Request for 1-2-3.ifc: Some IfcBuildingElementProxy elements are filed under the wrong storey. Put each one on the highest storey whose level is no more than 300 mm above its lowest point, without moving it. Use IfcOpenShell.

First a look at what the model holds.

```python
import ifcopenshell
import ifcopenshell.util.element
import ifcopenshell.util.placement

model = ifcopenshell.open("1-2-3.ifc")
print(model.schema)
for storey in model.by_type("IfcBuildingStorey"):
    level = ifcopenshell.util.placement.get_storey_elevation(storey)
    count = sum(e.is_a("IfcBuildingElementProxy") for e in ifcopenshell.util.element.get_contained(storey))
    print(storey.id(), storey.Name, round(level, 3), count, sep=" | ")
```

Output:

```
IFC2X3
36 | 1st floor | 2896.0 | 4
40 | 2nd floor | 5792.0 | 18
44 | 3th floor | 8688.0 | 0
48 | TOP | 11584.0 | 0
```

```python
import ifcopenshell
import ifcopenshell.api.spatial
import ifcopenshell.geom
import ifcopenshell.util.element
import ifcopenshell.util.placement
import ifcopenshell.util.shape
import ifcopenshell.util.unit

model = ifcopenshell.open("1-2-3.ifc")
unit_scale = ifcopenshell.util.unit.calculate_unit_scale(model)
settings = ifcopenshell.geom.settings()

levels = sorted(
    ((ifcopenshell.util.placement.get_storey_elevation(s) * unit_scale, s) for s in model.by_type("IfcBuildingStorey")),
    key=lambda pair: pair[0],
)

for e in model.by_type("IfcBuildingElementProxy"):
    current = e.ContainedInStructure[0].RelatingStructure if e.ContainedInStructure else None
    if current is None or not current.is_a("IfcBuildingStorey"):
        continue
    shape = ifcopenshell.geom.create_shape(settings, e)
    bottom = ifcopenshell.util.shape.get_shape_bottom_elevation(shape, shape.geometry)
    below = [s for level, s in levels if level <= bottom + 0.3]
    storey = below[-1] if below else levels[0][1]
    if storey != current:
        # assign_container keeps the world position.
        ifcopenshell.api.spatial.assign_container(model, products=[e], relating_structure=storey)
        print(e.id(), current.Name, "->", storey.Name)

model.write("1-2-3_v2.ifc")
```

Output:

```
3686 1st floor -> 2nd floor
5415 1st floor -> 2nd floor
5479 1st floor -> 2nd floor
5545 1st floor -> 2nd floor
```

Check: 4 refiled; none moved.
